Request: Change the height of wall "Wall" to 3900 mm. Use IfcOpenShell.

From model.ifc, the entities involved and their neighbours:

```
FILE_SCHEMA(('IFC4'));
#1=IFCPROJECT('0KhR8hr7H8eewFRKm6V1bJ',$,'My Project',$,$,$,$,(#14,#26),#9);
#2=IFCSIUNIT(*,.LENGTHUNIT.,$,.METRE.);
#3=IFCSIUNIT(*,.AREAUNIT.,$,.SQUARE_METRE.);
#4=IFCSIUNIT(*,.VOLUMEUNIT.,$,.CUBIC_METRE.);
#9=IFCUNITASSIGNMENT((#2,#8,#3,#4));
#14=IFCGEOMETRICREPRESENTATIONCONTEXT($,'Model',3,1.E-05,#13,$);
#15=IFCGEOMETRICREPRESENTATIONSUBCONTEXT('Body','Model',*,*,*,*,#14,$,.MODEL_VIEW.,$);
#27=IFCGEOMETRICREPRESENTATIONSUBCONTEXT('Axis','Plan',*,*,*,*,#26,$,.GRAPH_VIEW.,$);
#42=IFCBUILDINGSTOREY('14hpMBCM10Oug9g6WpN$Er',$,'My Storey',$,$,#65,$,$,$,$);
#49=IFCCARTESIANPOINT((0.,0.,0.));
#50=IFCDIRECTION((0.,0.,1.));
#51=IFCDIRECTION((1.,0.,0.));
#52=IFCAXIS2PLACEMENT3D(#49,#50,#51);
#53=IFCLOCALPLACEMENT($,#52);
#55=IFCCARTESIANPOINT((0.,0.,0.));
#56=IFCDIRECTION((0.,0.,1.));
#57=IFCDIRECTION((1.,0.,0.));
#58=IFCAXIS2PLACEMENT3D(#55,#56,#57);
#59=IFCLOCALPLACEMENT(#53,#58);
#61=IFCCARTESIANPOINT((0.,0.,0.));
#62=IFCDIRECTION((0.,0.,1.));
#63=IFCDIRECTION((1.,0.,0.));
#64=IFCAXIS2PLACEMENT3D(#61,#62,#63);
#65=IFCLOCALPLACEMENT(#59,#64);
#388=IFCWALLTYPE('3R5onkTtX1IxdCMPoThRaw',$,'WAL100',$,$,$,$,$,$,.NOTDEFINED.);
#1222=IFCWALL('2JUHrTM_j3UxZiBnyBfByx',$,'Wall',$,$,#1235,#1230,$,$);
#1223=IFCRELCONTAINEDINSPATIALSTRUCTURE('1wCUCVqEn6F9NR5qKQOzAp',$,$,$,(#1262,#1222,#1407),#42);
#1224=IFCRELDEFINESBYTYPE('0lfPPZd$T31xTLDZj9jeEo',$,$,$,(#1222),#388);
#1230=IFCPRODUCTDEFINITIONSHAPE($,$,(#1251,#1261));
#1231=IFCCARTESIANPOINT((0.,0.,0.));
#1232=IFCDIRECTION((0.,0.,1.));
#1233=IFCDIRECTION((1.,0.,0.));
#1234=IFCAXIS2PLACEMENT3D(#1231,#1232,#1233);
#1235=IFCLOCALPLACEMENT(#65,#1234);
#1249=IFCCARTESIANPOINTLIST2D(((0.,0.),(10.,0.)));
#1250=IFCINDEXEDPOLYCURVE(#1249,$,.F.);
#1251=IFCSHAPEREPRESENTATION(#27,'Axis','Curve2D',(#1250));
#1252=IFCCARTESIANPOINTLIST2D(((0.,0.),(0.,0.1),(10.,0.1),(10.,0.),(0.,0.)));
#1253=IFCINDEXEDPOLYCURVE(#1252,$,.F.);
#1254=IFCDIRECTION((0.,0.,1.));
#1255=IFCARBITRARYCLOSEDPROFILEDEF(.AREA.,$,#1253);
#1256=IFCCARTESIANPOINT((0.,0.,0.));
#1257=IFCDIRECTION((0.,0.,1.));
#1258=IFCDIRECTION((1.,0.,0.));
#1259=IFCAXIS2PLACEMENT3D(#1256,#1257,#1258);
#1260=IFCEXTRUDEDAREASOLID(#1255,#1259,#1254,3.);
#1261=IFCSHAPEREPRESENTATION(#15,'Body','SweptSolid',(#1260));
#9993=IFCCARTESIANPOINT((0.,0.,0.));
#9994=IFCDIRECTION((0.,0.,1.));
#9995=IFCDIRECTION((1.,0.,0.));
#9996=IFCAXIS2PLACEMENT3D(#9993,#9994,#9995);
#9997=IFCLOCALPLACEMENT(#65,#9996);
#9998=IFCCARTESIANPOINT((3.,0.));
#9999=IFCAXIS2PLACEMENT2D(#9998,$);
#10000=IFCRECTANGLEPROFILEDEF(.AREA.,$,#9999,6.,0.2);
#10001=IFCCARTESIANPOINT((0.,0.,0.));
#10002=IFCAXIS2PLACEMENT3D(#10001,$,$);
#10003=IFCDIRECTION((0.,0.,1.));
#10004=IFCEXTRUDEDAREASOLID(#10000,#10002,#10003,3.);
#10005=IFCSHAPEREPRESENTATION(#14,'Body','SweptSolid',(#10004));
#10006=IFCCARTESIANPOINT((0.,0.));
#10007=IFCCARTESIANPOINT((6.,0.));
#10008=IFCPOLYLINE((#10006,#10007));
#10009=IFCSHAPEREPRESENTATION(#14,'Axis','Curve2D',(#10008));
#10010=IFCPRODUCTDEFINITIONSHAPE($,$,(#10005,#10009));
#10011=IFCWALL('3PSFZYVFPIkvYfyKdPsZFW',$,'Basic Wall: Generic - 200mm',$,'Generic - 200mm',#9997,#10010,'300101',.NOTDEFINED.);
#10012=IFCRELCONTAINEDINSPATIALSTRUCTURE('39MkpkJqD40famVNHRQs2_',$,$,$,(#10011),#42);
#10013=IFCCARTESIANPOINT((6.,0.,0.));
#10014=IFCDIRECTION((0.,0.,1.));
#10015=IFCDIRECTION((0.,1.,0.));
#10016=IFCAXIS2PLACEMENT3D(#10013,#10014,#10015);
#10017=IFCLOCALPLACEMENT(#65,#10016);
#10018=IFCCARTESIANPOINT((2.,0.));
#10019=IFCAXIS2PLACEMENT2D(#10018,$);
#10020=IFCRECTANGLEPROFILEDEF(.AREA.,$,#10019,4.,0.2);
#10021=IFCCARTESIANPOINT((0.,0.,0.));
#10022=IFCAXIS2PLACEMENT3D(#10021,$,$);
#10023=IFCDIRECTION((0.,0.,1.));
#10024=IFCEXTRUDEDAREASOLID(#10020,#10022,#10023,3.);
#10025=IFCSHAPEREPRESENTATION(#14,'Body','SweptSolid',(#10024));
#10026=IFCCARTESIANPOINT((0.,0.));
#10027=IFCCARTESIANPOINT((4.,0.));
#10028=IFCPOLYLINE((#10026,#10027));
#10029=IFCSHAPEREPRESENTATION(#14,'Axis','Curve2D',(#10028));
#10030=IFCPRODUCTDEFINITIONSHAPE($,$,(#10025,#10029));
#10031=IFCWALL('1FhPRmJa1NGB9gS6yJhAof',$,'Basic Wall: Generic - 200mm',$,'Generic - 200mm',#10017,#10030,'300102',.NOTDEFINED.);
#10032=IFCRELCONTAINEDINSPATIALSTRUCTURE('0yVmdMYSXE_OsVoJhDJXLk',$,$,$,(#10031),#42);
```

```python
import ifcopenshell
import ifcopenshell.geom
import ifcopenshell.util.representation
import ifcopenshell.util.shape
import ifcopenshell.util.unit

model = ifcopenshell.open("model.ifc")
unit_scale = ifcopenshell.util.unit.calculate_unit_scale(model)
settings = ifcopenshell.geom.settings()


def volume(element):
    """Net volume in cubic metres, openings subtracted."""
    shape = ifcopenshell.geom.create_shape(settings, element)
    return ifcopenshell.util.shape.get_volume(shape.geometry)


wall = model.by_guid("2JUHrTM_j3UxZiBnyBfByx")
before = volume(wall)

body = ifcopenshell.util.representation.get_representation(wall, "Model", "Body")
solid = body.Items[0]
old_height = solid.Depth
solid.Depth = 3.9 / unit_scale
after = volume(wall)

print(f"height {old_height:g} -> {solid.Depth:g}, volume {before:.3f} -> {after:.3f} m3")

model.write("model_v2.ifc")
```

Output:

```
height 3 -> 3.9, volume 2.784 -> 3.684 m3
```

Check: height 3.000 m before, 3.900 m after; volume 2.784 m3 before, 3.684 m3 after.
